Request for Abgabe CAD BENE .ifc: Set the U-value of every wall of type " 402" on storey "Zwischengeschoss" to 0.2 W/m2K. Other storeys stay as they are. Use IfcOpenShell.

First a look at what the model holds.

```python
import ifcopenshell
import ifcopenshell.util.element

model = ifcopenshell.open("Abgabe CAD BENE .ifc")
print(model.schema)
storey = next(s for s in model.by_type("IfcBuildingStorey") if s.Name == "Zwischengeschoss")
walls = [e for e in ifcopenshell.util.element.get_decomposition(storey) if e.is_a("IfcWall")]
seen = {}
for e in walls:
    element_type = ifcopenshell.util.element.get_type(e)
    key = (element_type.Name if element_type != e and element_type else None, ifcopenshell.util.element.get_pset(e, "Pset_WallCommon", "ThermalTransmittance"))
    seen[key] = seen.get(key, 0) + 1
for (name, value), count in sorted(seen.items(), key=str):
    print(count, "x", name, "|", value)
```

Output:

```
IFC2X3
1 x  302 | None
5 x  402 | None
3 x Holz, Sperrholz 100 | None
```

```python
import ifcopenshell
import ifcopenshell.api.pset
import ifcopenshell.util.element

model = ifcopenshell.open("Abgabe CAD BENE .ifc")

storey = next(s for s in model.by_type("IfcBuildingStorey") if s.Name == "Zwischengeschoss")
walls = [e for e in ifcopenshell.util.element.get_decomposition(storey) if e.is_a("IfcWall")]

count = 0
for e in walls:
    element_type = ifcopenshell.util.element.get_type(e)
    if element_type in (None, e) or element_type.Name != " 402":
        continue
    # add_pset returns the element's existing set when there is one.
    pset = ifcopenshell.api.pset.add_pset(model, product=e, name="Pset_WallCommon")
    ifcopenshell.api.pset.edit_pset(model, pset=pset, properties={"ThermalTransmittance": 0.2})
    count += 1

print(count, "walls updated")

model.write("Abgabe CAD BENE _edited.ifc")
```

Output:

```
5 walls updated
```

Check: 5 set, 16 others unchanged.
